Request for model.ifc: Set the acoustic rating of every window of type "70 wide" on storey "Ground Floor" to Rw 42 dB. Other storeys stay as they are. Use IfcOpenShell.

First a look at what the model holds.

```python
import ifcopenshell
import ifcopenshell.util.element

model = ifcopenshell.open("model.ifc")
print(model.schema)
storey = next(s for s in model.by_type("IfcBuildingStorey") if s.Name == "Ground Floor")
windows = [e for e in ifcopenshell.util.element.get_decomposition(storey) if e.is_a("IfcWindow")]
seen = {}
for e in windows:
    element_type = ifcopenshell.util.element.get_type(e)
    key = (element_type.Name if element_type != e and element_type else None, ifcopenshell.util.element.get_pset(e, "Pset_WindowCommon", "AcousticRating"))
    seen[key] = seen.get(key, 0) + 1
for (name, value), count in sorted(seen.items(), key=str):
    print(count, "x", name, "|", value)
```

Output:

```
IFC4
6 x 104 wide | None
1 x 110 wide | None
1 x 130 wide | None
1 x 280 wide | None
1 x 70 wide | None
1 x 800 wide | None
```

```python
import ifcopenshell
import ifcopenshell.api.pset
import ifcopenshell.util.element

model = ifcopenshell.open("model.ifc")

storey = next(s for s in model.by_type("IfcBuildingStorey") if s.Name == "Ground Floor")
windows = [e for e in ifcopenshell.util.element.get_decomposition(storey) if e.is_a("IfcWindow")]

count = 0
for e in windows:
    element_type = ifcopenshell.util.element.get_type(e)
    if element_type in (None, e) or element_type.Name != "70 wide":
        continue
    # add_pset returns the element's existing set when there is one.
    pset = ifcopenshell.api.pset.add_pset(model, product=e, name="Pset_WindowCommon")
    ifcopenshell.api.pset.edit_pset(model, pset=pset, properties={"AcousticRating": "Rw 42 dB"})
    count += 1

print(count, "windows updated")

model.write("model_rev.ifc")
```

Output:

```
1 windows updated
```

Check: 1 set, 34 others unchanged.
